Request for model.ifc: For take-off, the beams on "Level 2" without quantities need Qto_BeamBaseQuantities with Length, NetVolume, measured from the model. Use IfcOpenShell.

First a look at what the model holds.

```python
import ifcopenshell
import ifcopenshell.util.element
import ifcopenshell.util.unit

model = ifcopenshell.open("model.ifc")
print(model.schema)
for unit_type in ("LENGTHUNIT", "AREAUNIT", "VOLUMEUNIT"):
    print(unit_type, ifcopenshell.util.unit.calculate_unit_scale(model, unit_type))
storey = next(s for s in model.by_type("IfcBuildingStorey") if s.Name == "Level 2")
beams = [e for e in ifcopenshell.util.element.get_decomposition(storey) if e.is_a("IfcBeam")]
for e in sorted(beams, key=lambda e: e.id()):
    print(e.id(), e.is_a(), e.Name, list(ifcopenshell.util.element.get_psets(e, qtos_only=True)), sep=" | ")
```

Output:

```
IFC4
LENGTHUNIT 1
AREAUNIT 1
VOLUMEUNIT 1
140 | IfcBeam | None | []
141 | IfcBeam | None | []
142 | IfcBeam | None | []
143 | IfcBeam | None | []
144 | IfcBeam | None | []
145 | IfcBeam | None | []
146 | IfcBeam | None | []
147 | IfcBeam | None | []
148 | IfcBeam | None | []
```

```python
import ifcopenshell
import ifcopenshell.api.pset
import ifcopenshell.geom
import ifcopenshell.util.element
import ifcopenshell.util.shape
import ifcopenshell.util.unit

model = ifcopenshell.open("model.ifc")
unit_scale = ifcopenshell.util.unit.calculate_unit_scale(model)
volume_scale = ifcopenshell.util.unit.calculate_unit_scale(model, "VOLUMEUNIT")
settings = ifcopenshell.geom.settings()

storey = next(s for s in model.by_type("IfcBuildingStorey") if s.Name == "Level 2")
beams = [e for e in ifcopenshell.util.element.get_decomposition(storey) if e.is_a("IfcBeam")]

for e in sorted(beams, key=lambda e: e.id()):
    if ifcopenshell.util.element.get_psets(e, qtos_only=True, should_inherit=False):
        continue
    # Geometry comes back in metres, in the element's own axes.
    shape = ifcopenshell.geom.create_shape(settings, e)
    values = {
        "Length": ifcopenshell.util.shape.get_max_xyz(shape.geometry) / unit_scale,
        "NetVolume": ifcopenshell.util.shape.get_volume(shape.geometry) / volume_scale,
    }
    qto = ifcopenshell.api.pset.add_qto(model, product=e, name="Qto_BeamBaseQuantities")
    ifcopenshell.api.pset.edit_qto(model, qto=qto, properties=values)
    print(e.id(), {k: round(v, 3) for k, v in values.items()})

model.write("model_rev.ifc")
```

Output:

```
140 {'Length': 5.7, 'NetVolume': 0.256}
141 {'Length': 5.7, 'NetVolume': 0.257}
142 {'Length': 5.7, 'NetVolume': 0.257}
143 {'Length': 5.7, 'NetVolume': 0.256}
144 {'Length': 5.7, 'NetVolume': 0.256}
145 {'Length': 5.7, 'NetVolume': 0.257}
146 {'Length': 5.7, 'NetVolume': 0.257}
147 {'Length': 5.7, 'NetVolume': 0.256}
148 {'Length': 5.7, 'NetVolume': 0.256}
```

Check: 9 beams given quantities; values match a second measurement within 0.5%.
